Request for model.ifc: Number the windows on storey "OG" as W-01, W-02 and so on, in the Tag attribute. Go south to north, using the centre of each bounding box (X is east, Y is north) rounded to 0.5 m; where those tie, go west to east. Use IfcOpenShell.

First a look at what the model holds.

```python
import ifcopenshell
import ifcopenshell.util.element
import ifcopenshell.util.placement

model = ifcopenshell.open("model.ifc")
print(model.schema)
storey = next(s for s in model.by_type("IfcBuildingStorey") if s.Name == "OG")
windows = [e for e in ifcopenshell.util.element.get_decomposition(storey) if e.is_a("IfcWindow")]
for e in sorted(windows, key=lambda e: e.id()):
    origin = ifcopenshell.util.placement.get_local_placement(e.ObjectPlacement)[:3, 3]
    print(e.id(), e.Tag, e.Name, origin.round(2) + 0.0, sep=" | ")
```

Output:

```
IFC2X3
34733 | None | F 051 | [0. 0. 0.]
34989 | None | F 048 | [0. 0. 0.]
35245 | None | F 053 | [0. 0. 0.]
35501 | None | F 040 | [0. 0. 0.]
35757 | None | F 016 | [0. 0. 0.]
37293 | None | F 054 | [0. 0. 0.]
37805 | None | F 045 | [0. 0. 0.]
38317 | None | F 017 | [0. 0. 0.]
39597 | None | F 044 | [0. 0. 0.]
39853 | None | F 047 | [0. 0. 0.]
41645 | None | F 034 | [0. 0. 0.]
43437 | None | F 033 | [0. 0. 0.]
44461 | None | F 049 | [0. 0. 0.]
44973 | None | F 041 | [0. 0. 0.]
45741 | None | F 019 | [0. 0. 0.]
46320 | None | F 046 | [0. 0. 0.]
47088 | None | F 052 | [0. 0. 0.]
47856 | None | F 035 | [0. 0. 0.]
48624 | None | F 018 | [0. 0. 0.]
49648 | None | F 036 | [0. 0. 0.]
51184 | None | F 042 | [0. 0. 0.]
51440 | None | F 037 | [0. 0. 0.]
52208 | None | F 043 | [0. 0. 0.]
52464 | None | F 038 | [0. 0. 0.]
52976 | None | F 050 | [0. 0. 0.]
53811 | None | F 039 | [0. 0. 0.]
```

```python
import ifcopenshell
import ifcopenshell.geom
import ifcopenshell.util.element
import ifcopenshell.util.shape

model = ifcopenshell.open("model.ifc")
settings = ifcopenshell.geom.settings()
settings.set("use-world-coords", True)


def centre(element):
    shape = ifcopenshell.geom.create_shape(settings, element)
    return ifcopenshell.util.shape.get_bbox_centroid(shape.geometry)


storey = next(s for s in model.by_type("IfcBuildingStorey") if s.Name == "OG")
windows = [e for e in ifcopenshell.util.element.get_decomposition(storey) if e.is_a("IfcWindow")]

# Insertion points can sit at a corner or the storey origin, so sort by the geometry (in metres).
centres = {e: centre(e) for e in windows}
windows.sort(key=lambda e: (round(centres[e][1] / 0.5), centres[e][0]))

for i, e in enumerate(windows, start=1):
    number = f"W-{i:02d}"
    e.Tag = number
    print(e.id(), number)

model.write("model-out.ifc")
```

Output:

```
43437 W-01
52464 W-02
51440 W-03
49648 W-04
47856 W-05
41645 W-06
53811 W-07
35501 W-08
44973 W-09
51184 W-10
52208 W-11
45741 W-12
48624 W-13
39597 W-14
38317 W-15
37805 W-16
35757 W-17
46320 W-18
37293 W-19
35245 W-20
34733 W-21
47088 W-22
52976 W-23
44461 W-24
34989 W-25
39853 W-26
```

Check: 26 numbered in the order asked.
